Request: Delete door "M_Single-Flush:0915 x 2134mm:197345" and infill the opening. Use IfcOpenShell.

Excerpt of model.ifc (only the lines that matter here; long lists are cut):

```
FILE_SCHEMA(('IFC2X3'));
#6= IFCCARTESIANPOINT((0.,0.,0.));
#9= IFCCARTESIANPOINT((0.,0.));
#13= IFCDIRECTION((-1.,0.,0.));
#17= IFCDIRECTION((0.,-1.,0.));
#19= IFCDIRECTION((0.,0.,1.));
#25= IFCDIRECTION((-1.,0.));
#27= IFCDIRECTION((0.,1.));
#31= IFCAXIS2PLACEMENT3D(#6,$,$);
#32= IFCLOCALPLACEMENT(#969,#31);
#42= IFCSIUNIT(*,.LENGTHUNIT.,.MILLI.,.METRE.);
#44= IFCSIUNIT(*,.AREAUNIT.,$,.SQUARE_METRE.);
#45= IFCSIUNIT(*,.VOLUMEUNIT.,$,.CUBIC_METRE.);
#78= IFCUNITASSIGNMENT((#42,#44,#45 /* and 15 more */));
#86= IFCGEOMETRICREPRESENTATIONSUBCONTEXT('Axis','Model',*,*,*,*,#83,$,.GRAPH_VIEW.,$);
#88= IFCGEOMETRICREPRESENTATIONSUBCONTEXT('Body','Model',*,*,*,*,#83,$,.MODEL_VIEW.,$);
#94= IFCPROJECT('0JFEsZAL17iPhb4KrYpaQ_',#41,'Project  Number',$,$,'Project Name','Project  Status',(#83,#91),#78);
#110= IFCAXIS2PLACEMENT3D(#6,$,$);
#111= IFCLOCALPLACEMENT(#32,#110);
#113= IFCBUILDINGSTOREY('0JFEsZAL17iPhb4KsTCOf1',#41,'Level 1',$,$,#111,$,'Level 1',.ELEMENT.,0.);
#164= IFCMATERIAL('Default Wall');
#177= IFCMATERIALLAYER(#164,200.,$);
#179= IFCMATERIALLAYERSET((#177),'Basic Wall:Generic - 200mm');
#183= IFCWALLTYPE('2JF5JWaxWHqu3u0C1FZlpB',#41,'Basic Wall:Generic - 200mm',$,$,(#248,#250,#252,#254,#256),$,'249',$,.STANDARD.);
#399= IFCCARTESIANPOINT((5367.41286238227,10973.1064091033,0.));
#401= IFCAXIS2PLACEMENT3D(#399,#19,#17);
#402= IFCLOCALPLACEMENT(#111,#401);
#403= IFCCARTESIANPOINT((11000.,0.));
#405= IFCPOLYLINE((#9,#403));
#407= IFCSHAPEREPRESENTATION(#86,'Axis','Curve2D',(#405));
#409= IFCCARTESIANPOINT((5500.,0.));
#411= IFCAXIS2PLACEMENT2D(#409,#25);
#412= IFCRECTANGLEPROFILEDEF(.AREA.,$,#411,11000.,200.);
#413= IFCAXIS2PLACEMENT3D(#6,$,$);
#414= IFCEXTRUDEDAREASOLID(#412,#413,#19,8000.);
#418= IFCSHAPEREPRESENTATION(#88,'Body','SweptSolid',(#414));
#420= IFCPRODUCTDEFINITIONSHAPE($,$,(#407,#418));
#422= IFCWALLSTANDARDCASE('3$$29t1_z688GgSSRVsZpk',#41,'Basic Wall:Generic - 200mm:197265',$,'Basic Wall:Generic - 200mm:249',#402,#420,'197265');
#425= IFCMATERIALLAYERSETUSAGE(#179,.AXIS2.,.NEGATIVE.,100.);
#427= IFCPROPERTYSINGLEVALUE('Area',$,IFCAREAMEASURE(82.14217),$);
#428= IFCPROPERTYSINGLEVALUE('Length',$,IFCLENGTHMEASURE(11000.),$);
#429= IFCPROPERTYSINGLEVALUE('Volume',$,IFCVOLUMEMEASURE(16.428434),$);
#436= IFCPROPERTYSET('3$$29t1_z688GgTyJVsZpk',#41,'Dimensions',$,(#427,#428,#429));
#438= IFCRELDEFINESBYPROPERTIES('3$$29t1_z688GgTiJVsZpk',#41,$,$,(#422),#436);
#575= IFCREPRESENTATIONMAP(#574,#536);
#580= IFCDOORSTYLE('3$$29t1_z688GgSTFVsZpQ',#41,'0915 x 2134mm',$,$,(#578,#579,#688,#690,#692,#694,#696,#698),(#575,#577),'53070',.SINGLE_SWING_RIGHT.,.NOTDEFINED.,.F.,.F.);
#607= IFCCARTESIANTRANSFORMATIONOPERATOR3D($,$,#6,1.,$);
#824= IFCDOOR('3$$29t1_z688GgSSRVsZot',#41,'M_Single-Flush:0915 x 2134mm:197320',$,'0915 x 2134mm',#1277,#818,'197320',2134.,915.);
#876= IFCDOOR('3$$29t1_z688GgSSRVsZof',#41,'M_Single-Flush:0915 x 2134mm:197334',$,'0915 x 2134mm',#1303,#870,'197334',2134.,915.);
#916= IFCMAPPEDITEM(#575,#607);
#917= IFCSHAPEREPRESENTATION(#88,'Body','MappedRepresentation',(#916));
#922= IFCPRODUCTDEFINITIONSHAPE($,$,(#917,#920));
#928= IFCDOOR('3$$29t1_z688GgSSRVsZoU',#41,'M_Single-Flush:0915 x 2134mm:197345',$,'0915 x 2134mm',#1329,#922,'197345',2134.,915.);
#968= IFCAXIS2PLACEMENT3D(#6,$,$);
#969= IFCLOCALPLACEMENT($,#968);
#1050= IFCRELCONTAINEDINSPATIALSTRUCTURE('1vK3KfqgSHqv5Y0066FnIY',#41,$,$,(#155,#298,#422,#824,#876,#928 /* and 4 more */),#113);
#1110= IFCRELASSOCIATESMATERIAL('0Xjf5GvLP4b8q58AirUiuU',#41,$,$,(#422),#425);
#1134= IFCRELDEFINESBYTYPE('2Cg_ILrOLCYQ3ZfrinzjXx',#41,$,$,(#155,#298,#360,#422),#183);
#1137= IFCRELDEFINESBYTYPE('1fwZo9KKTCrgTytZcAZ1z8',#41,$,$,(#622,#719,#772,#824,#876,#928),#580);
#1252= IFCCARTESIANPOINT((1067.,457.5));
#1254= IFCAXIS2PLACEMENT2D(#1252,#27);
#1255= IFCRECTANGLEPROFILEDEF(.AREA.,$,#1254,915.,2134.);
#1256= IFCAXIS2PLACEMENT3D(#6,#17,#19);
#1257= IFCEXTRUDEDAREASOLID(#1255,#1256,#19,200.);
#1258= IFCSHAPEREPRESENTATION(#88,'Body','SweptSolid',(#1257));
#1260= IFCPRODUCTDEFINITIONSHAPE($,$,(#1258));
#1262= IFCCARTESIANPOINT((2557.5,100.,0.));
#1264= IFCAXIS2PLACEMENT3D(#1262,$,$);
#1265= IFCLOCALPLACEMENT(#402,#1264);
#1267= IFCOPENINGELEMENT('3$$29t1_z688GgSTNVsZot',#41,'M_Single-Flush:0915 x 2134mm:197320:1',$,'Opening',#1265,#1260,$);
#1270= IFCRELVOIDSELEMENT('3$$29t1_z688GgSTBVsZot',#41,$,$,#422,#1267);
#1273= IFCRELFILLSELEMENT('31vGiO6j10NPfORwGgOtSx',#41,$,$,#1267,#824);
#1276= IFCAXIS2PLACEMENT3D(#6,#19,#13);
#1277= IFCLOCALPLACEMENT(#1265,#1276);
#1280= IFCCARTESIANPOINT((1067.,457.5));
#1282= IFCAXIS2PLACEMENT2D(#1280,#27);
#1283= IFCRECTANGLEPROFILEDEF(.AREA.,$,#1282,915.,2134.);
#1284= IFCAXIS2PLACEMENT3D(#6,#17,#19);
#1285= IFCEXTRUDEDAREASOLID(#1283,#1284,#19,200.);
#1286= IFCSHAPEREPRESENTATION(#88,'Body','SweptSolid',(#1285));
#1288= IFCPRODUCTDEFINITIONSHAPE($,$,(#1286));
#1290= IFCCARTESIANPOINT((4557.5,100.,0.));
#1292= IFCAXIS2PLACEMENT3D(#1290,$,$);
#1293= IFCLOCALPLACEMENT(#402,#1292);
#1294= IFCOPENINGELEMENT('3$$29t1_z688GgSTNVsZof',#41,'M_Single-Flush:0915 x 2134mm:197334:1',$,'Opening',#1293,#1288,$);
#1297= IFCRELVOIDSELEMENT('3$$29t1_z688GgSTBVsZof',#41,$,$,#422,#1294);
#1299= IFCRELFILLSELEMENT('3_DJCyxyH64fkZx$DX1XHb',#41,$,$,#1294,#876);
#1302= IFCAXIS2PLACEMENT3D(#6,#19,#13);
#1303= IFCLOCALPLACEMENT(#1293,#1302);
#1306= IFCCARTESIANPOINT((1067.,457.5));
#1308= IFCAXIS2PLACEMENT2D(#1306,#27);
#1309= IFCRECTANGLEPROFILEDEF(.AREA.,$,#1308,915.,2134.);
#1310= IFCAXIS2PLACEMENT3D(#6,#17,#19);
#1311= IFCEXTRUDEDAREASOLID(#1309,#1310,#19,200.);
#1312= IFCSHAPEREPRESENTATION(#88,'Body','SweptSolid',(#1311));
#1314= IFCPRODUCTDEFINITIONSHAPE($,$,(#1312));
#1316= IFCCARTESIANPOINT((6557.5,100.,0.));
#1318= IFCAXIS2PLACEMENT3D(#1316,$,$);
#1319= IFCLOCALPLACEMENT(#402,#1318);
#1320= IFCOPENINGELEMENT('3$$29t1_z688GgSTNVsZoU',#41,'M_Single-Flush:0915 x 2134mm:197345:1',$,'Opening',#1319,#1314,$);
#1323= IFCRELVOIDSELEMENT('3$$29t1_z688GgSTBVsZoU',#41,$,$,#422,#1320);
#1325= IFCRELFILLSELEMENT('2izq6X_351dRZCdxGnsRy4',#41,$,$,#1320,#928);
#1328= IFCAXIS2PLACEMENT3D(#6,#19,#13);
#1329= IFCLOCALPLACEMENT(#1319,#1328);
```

```python
import ifcopenshell
import ifcopenshell.api.feature
import ifcopenshell.api.pset
import ifcopenshell.api.root
import ifcopenshell.geom
import ifcopenshell.util.element
import ifcopenshell.util.shape
import ifcopenshell.util.unit

model = ifcopenshell.open("model.ifc")
area_scale = ifcopenshell.util.unit.calculate_unit_scale(model, "AREAUNIT")
volume_scale = ifcopenshell.util.unit.calculate_unit_scale(model, "VOLUMEUNIT")
settings = ifcopenshell.geom.settings()


def volume(element):
    """Net volume in cubic metres, openings subtracted."""
    shape = ifcopenshell.geom.create_shape(settings, element)
    return ifcopenshell.util.shape.get_volume(shape.geometry)


door = model.by_guid("3$$29t1_z688GgSSRVsZoU")
opening = door.FillsVoids[0].RelatingOpeningElement
wall = opening.VoidsElements[0].RelatingBuildingElement
before = volume(wall)

ifcopenshell.api.root.remove_product(model, product=door)
ifcopenshell.api.feature.remove_feature(model, feature=opening)

after = volume(wall)
thickness = 0.2  # wall thickness in metres

# Update the wall's stored quantities.
pset = model.by_id(ifcopenshell.util.element.get_pset(wall, "Dimensions", should_inherit=False)["id"])
ifcopenshell.api.pset.edit_pset(model, pset=pset, properties={
    "Area": model.create_entity("IfcAreaMeasure", after / thickness / area_scale),
    "Volume": model.create_entity("IfcVolumeMeasure", after / volume_scale),
})

print(f"wall volume {before:.3f} -> {after:.3f} m3")

model.write("model_rev.ifc")
```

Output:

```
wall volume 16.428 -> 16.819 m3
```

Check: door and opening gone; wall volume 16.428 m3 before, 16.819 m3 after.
